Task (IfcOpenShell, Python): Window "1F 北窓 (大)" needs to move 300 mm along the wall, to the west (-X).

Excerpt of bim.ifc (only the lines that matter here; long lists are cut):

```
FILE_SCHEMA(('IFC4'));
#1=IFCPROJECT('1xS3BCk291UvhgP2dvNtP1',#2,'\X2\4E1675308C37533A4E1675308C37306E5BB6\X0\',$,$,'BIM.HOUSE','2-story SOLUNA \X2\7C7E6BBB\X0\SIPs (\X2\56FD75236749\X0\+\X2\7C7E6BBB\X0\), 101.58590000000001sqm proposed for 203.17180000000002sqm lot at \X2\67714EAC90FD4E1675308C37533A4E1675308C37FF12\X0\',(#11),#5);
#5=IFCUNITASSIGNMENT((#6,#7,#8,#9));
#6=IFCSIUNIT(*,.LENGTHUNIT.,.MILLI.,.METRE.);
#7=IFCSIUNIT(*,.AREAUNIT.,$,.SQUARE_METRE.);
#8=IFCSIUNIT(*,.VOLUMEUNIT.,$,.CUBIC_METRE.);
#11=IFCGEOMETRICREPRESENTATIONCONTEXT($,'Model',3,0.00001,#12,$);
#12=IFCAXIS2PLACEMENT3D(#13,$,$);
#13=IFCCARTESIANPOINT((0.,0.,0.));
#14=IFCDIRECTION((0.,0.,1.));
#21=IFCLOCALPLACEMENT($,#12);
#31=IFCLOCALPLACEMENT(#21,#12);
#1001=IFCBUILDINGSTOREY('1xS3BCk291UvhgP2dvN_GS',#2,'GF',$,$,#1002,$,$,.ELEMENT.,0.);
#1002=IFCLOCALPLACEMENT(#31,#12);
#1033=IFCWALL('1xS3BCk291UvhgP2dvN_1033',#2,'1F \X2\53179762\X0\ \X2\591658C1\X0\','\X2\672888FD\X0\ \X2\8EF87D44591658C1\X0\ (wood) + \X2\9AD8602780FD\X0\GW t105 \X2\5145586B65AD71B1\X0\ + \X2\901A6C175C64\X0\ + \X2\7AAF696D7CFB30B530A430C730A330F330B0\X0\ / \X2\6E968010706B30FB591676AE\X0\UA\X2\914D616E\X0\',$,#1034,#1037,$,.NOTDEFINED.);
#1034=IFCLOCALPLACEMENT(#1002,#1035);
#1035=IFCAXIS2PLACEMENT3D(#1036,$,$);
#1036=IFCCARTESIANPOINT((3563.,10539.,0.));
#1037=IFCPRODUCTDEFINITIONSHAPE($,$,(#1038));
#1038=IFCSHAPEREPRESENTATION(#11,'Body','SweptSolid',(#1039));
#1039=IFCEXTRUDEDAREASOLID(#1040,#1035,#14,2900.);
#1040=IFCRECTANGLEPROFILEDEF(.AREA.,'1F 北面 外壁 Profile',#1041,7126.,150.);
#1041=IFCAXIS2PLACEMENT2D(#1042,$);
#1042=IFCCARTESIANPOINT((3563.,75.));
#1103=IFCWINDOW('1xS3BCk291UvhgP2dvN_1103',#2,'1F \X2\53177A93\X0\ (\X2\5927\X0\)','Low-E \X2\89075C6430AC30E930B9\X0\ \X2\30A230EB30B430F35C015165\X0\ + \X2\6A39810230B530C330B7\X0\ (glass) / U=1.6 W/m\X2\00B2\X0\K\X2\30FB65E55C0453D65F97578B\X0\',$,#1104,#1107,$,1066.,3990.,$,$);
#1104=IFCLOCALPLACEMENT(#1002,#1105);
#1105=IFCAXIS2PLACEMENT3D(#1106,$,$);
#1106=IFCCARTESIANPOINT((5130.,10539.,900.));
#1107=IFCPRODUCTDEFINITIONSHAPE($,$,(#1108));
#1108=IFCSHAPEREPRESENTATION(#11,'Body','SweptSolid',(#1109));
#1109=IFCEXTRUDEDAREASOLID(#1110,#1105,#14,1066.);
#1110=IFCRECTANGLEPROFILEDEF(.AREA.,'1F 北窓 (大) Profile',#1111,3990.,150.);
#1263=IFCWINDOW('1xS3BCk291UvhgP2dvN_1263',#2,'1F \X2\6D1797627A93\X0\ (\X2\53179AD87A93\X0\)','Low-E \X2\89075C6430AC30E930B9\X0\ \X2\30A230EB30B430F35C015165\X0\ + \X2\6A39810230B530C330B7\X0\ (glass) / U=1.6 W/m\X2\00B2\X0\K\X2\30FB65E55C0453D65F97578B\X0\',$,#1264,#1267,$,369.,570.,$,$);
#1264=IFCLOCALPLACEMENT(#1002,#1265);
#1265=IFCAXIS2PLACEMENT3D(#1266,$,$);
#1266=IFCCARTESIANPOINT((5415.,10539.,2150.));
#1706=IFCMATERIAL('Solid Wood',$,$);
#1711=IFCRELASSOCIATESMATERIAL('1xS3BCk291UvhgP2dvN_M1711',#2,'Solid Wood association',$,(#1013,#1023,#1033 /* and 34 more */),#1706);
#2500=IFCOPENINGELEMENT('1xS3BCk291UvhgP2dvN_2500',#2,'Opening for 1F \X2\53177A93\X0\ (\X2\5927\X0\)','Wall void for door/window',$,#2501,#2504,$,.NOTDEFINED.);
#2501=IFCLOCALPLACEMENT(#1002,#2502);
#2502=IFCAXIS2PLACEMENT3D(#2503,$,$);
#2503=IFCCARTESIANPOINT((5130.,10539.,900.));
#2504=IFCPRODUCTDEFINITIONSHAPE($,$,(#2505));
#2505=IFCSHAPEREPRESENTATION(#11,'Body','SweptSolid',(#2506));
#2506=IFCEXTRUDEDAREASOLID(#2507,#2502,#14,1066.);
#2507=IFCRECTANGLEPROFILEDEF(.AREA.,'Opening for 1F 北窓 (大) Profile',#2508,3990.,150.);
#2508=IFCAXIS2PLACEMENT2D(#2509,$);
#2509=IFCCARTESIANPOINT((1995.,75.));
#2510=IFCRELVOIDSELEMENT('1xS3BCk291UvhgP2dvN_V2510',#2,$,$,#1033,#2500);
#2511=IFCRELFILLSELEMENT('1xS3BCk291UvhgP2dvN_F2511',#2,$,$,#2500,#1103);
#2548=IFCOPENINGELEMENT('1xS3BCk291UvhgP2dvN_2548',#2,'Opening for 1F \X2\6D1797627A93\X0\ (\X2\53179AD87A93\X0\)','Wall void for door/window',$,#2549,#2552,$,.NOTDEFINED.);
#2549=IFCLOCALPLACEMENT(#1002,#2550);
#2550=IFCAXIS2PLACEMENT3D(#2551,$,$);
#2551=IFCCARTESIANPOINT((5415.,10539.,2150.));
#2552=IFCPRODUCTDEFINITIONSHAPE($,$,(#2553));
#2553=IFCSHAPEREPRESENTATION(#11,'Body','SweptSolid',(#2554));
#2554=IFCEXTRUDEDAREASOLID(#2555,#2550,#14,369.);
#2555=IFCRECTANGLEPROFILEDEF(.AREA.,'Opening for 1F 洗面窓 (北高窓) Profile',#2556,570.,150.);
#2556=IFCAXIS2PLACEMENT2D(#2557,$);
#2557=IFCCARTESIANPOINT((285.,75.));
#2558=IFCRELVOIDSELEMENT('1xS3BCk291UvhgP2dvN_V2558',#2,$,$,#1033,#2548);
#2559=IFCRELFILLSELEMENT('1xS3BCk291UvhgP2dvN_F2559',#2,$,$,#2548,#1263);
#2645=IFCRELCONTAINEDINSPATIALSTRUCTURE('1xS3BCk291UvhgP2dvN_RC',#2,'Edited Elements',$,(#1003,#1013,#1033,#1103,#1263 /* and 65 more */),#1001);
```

```python
import ifcopenshell
import ifcopenshell.api.geometry
import ifcopenshell.util.placement
import ifcopenshell.util.unit

model = ifcopenshell.open("bim.ifc")
unit_scale = ifcopenshell.util.unit.calculate_unit_scale(model)

window = model.by_guid("1xS3BCk291UvhgP2dvN_1103")
opening = window.FillsVoids[0].RelatingOpeningElement
wall = opening.VoidsElements[0].RelatingBuildingElement

wall_matrix = ifcopenshell.util.placement.get_local_placement(wall.ObjectPlacement)
shift = wall_matrix[:3, 0] * -0.3 / unit_scale
before = ifcopenshell.util.placement.get_local_placement(window.ObjectPlacement)[:3, 3].copy()

# The window is not placed relative to its opening, so move both.
for product in (opening, window):
    matrix = ifcopenshell.util.placement.get_local_placement(product.ObjectPlacement)
    matrix[:3, 3] += shift
    ifcopenshell.api.geometry.edit_object_placement(model, product=product, matrix=matrix, is_si=False)

after = ifcopenshell.util.placement.get_local_placement(window.ObjectPlacement)[:3, 3]
print("window moved by", (after - before).round(3) + 0.0)

model.write("bim_v2.ifc")
```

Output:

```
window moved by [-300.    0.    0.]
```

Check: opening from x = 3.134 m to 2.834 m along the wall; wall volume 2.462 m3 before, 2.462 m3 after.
